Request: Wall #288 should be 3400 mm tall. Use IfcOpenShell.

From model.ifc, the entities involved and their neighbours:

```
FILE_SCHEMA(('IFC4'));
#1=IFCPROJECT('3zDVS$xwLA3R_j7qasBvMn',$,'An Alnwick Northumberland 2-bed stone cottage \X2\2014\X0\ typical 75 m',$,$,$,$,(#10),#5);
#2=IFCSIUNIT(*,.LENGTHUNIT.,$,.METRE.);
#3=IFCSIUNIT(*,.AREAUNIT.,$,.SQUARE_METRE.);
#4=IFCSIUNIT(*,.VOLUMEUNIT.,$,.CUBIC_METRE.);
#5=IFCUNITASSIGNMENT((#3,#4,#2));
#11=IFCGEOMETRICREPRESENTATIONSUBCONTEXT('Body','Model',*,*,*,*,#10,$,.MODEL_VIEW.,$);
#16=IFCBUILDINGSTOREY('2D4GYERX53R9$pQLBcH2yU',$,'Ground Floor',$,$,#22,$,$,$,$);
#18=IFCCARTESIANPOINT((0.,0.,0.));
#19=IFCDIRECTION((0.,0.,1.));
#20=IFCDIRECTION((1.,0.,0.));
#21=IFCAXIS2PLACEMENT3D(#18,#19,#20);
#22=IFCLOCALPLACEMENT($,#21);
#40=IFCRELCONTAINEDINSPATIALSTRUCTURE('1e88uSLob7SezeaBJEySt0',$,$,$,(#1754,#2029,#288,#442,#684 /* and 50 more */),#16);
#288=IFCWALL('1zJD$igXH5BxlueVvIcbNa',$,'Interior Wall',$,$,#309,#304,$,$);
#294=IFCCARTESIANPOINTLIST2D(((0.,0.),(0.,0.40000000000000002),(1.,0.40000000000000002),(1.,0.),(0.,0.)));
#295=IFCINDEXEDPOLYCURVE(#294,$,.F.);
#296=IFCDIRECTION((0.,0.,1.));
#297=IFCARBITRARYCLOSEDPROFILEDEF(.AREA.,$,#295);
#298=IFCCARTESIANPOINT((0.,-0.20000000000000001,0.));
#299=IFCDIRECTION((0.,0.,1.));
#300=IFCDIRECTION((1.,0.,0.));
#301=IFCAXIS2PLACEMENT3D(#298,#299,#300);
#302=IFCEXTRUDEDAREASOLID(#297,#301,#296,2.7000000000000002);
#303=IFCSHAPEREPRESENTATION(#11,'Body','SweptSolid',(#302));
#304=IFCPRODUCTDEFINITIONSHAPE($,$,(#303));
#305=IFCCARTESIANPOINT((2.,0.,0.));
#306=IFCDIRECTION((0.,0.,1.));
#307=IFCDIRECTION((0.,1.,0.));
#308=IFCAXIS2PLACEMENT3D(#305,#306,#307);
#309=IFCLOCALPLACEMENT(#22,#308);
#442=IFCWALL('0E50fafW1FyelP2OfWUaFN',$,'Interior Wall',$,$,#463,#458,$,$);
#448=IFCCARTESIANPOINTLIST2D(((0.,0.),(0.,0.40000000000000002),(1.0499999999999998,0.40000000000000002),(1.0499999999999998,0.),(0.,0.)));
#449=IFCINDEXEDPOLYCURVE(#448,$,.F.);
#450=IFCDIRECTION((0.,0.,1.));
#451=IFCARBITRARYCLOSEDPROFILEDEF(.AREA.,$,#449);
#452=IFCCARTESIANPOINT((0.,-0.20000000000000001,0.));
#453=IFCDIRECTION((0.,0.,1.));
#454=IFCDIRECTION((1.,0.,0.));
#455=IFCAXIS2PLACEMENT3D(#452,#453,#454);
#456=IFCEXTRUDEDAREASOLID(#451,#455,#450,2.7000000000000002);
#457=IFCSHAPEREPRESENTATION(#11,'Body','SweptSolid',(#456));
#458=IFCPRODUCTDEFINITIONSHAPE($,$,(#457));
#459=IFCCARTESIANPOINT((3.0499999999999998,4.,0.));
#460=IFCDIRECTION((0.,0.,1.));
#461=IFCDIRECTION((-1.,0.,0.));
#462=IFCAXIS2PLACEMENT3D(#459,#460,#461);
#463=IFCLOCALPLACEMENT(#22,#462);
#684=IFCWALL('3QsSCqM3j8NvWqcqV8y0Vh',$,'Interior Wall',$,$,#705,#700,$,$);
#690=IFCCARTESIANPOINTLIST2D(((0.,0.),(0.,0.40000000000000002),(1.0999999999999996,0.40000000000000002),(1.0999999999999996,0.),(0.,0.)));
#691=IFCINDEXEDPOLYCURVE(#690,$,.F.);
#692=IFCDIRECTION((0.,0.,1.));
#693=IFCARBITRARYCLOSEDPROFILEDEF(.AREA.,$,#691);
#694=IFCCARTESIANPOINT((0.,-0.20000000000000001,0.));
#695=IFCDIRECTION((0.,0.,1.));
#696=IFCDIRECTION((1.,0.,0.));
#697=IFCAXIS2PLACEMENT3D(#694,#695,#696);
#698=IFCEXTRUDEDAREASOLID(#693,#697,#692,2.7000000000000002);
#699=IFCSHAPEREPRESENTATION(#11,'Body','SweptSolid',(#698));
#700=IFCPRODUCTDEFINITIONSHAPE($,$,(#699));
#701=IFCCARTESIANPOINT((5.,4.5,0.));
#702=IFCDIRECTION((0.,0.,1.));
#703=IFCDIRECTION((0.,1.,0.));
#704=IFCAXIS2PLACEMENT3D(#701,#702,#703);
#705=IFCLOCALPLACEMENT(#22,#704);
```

```python
import ifcopenshell
import ifcopenshell.geom
import ifcopenshell.util.representation
import ifcopenshell.util.shape

model = ifcopenshell.open("model.ifc")
settings = ifcopenshell.geom.settings()


def volume(element):
    """Net volume in cubic metres, openings subtracted."""
    shape = ifcopenshell.geom.create_shape(settings, element)
    return ifcopenshell.util.shape.get_volume(shape.geometry)


wall = model.by_id(288)
before = volume(wall)

body = ifcopenshell.util.representation.get_representation(wall, "Model", "Body")
solid = body.Items[0]
old_height = solid.Depth
solid.Depth = 3.4
after = volume(wall)

print(f"height {old_height:g} -> {solid.Depth:g}, volume {before:.3f} -> {after:.3f} m3")

model.write("model_v2.ifc")
```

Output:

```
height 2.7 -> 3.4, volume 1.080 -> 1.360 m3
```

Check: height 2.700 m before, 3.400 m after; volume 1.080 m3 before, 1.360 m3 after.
